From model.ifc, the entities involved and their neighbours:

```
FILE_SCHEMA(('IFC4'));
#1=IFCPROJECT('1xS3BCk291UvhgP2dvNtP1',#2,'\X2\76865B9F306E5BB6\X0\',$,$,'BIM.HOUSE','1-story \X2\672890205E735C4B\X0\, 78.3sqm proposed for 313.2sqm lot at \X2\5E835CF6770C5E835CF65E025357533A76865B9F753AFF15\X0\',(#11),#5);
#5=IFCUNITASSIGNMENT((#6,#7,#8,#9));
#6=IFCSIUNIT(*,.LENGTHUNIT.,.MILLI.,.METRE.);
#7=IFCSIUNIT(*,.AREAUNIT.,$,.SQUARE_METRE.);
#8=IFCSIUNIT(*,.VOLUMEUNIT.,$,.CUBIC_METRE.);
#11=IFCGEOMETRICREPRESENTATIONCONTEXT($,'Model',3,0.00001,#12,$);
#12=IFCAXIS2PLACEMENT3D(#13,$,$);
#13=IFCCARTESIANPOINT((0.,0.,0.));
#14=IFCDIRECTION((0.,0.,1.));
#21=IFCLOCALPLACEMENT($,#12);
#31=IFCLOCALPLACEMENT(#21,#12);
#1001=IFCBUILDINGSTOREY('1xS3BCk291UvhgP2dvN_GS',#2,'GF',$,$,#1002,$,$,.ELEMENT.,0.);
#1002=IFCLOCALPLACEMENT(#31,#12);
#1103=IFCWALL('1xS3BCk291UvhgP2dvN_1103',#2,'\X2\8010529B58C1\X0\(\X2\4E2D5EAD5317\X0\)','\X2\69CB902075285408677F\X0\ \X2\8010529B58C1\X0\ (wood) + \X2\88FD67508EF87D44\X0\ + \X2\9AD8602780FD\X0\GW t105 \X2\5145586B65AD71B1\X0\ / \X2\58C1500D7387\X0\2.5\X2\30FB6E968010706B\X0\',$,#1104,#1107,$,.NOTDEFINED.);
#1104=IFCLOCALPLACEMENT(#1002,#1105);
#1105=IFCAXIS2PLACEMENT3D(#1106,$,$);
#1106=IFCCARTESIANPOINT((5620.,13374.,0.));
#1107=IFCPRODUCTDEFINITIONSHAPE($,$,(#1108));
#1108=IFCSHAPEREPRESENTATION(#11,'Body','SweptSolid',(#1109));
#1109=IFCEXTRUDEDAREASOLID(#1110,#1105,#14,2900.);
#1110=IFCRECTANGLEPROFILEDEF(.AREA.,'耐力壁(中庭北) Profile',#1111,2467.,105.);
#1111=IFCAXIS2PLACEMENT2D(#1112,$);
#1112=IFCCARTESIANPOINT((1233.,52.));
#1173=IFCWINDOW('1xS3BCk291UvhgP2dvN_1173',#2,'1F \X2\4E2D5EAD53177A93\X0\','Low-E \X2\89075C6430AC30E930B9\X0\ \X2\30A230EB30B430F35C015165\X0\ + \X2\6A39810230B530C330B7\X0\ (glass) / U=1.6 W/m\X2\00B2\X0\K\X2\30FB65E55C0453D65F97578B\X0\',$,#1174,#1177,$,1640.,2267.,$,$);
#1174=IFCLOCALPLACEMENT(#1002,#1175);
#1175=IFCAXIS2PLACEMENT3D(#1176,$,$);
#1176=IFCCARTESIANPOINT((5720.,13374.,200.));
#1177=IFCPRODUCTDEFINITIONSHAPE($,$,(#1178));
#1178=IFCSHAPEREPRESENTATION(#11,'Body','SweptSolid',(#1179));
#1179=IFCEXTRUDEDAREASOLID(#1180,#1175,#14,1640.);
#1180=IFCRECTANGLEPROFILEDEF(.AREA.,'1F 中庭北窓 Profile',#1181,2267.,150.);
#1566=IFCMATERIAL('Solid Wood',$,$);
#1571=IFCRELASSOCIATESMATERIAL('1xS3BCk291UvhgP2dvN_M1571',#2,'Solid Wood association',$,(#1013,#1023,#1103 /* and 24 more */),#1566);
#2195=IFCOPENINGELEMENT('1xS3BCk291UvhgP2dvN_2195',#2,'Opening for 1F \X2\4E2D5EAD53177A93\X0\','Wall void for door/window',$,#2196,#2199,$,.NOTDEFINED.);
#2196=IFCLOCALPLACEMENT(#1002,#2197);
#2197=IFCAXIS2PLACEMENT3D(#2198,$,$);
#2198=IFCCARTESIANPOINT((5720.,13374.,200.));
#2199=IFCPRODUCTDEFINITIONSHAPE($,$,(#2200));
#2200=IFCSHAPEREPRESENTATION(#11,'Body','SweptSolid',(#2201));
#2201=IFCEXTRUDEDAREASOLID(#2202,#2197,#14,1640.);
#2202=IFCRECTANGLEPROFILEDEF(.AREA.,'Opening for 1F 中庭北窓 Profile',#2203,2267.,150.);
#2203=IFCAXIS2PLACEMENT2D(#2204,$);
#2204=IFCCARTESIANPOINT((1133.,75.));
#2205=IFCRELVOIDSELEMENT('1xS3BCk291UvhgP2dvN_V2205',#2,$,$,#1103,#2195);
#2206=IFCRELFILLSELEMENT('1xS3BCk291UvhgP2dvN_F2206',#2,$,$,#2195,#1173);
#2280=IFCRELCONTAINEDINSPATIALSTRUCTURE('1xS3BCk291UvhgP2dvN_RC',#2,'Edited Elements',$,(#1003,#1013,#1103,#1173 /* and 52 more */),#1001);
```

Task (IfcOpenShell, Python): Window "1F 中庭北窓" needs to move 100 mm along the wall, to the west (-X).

```python
import ifcopenshell
import ifcopenshell.api.geometry
import ifcopenshell.util.placement

model = ifcopenshell.open("model.ifc")

window = model.by_id(1173)
opening = window.FillsVoids[0].RelatingOpeningElement
wall = opening.VoidsElements[0].RelatingBuildingElement

wall_matrix = ifcopenshell.util.placement.get_local_placement(wall.ObjectPlacement)
shift = wall_matrix[:3, 0] * -100.0
before = ifcopenshell.util.placement.get_local_placement(window.ObjectPlacement)[:3, 3].copy()

# The window is not placed relative to its opening, so move both.
for product in (opening, window):
    matrix = ifcopenshell.util.placement.get_local_placement(product.ObjectPlacement)
    matrix[:3, 3] += shift
    ifcopenshell.api.geometry.edit_object_placement(model, product=product, matrix=matrix, is_si=False)

after = ifcopenshell.util.placement.get_local_placement(window.ObjectPlacement)[:3, 3]
print("window moved by", (after - before).round(3) + 0.0)

model.write("model_rev.ifc")
```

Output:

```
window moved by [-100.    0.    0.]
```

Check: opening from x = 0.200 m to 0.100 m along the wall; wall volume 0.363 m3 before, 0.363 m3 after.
